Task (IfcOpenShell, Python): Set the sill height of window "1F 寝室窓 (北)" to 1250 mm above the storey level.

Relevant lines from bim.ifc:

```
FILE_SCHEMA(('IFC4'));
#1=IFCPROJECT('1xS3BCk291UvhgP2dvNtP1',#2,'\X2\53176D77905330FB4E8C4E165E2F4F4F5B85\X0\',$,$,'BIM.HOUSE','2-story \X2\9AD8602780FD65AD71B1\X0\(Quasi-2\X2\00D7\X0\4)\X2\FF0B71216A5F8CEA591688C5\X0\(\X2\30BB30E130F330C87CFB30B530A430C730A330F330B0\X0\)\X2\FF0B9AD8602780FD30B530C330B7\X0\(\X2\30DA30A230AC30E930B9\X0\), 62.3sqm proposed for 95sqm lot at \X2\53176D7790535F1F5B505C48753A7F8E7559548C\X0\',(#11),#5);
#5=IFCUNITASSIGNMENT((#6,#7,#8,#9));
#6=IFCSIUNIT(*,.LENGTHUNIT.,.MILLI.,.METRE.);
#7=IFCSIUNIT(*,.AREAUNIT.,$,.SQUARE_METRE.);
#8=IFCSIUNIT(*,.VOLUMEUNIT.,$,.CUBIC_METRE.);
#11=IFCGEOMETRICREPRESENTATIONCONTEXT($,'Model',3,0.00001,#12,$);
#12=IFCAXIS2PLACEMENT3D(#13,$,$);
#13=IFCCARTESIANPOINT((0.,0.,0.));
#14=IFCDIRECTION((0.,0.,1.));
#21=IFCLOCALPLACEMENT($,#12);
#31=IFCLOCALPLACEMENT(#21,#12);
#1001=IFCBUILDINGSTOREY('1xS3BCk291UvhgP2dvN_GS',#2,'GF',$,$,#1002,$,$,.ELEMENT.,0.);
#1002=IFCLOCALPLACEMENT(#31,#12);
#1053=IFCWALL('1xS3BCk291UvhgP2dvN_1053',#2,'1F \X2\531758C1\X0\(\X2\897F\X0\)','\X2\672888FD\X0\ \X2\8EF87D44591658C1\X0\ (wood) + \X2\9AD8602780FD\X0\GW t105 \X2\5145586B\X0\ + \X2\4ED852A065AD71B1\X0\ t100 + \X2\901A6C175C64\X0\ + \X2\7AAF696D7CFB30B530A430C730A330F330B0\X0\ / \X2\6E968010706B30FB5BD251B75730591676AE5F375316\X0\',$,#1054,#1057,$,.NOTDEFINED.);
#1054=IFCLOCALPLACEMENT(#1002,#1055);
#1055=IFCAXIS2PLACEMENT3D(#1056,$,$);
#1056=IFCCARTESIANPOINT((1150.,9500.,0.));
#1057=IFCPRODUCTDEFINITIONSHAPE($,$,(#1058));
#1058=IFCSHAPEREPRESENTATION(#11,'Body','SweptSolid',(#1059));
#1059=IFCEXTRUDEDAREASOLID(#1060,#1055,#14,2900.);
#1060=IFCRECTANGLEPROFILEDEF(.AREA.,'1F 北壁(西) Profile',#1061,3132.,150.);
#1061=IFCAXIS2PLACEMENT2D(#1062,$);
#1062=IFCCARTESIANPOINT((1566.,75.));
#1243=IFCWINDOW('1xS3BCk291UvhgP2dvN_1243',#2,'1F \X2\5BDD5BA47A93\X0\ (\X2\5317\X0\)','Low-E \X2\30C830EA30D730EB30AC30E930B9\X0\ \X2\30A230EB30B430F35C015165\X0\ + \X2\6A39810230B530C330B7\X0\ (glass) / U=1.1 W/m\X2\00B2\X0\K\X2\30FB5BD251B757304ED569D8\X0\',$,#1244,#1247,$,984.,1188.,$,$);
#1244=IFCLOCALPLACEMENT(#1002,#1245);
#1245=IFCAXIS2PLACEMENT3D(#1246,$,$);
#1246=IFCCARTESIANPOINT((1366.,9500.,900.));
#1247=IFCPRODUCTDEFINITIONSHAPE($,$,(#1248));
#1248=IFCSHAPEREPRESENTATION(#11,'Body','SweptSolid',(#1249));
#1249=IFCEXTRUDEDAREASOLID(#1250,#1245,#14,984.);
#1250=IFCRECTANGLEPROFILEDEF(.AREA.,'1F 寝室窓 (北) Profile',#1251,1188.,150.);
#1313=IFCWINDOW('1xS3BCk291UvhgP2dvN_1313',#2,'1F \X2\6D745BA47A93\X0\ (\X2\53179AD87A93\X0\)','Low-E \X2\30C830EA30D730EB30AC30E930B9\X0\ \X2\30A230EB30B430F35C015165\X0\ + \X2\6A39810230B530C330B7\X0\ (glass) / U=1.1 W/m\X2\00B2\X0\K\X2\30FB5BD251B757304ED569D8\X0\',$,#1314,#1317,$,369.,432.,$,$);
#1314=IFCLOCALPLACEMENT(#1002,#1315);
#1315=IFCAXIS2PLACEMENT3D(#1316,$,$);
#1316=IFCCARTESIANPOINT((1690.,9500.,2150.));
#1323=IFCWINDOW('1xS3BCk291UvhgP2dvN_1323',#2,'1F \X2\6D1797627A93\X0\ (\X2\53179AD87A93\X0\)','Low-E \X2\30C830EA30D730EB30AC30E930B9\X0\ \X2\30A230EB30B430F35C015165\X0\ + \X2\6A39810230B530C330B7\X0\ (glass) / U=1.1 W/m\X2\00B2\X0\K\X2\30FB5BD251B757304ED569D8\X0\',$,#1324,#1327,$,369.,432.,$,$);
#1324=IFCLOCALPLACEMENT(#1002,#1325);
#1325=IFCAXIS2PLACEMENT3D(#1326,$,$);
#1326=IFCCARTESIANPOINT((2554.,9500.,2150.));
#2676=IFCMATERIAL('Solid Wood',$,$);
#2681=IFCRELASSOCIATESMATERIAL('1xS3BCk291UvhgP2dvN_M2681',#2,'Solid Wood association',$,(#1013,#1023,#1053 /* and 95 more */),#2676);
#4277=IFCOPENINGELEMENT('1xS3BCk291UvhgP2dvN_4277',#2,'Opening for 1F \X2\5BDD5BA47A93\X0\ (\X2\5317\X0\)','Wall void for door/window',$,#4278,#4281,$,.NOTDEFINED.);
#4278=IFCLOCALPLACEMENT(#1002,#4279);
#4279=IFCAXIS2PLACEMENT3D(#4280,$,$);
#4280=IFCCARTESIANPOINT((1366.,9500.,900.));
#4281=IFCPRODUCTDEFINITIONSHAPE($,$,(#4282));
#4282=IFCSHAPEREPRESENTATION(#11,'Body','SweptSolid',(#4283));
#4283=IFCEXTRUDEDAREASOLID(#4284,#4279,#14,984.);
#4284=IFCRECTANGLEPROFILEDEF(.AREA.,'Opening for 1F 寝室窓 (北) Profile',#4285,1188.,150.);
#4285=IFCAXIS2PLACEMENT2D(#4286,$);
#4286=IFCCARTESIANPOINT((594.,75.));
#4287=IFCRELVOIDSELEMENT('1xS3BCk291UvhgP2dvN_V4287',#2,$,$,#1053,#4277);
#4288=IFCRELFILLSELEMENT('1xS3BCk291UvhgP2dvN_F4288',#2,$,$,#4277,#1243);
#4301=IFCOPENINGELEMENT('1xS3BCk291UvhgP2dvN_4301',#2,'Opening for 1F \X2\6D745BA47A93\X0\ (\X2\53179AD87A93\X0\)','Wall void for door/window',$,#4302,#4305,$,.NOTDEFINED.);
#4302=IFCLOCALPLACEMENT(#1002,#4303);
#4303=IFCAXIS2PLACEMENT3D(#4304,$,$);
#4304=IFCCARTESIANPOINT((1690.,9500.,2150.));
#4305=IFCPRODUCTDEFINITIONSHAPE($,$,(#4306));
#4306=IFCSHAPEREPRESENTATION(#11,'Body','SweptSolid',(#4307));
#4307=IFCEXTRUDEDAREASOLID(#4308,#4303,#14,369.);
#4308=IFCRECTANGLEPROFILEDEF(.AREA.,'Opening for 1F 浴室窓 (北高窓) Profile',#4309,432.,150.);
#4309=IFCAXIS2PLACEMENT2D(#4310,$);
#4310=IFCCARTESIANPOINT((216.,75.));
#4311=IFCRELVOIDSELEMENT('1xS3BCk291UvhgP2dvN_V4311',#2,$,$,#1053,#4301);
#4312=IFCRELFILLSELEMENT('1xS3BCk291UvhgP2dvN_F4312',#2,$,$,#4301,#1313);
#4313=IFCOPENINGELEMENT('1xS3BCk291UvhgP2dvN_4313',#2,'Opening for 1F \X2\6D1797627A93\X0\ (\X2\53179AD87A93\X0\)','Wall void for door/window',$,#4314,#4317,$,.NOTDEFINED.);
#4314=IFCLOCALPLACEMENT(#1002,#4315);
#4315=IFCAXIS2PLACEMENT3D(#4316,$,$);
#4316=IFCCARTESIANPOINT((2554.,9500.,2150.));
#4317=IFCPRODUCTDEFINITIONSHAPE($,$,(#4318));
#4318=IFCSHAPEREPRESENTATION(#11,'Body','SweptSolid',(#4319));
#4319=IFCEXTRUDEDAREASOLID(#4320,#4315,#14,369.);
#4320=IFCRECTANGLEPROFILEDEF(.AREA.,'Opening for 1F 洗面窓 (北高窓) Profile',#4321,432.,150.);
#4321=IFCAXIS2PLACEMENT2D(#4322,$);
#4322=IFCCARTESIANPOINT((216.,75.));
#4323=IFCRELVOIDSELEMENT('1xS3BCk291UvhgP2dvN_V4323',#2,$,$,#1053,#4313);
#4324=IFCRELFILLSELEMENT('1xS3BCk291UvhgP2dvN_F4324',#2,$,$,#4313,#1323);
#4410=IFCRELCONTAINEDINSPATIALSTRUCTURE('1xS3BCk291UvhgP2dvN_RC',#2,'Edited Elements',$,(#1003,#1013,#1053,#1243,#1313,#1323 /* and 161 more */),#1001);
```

```python
import numpy as np
import ifcopenshell
import ifcopenshell.api.geometry
import ifcopenshell.geom
import ifcopenshell.util.element
import ifcopenshell.util.placement
import ifcopenshell.util.shape
import ifcopenshell.util.unit

model = ifcopenshell.open("bim.ifc")
unit_scale = ifcopenshell.util.unit.calculate_unit_scale(model)

window = model.by_id(1243)
opening = window.FillsVoids[0].RelatingOpeningElement
storey = ifcopenshell.util.element.get_container(window, ifc_class="IfcBuildingStorey")
level = ifcopenshell.util.placement.get_local_placement(storey.ObjectPlacement)[2, 3]

# The opening's origin need not be at the sill, so measure its lowest point.
shape = ifcopenshell.geom.create_shape(ifcopenshell.geom.settings(), opening)
bottom = ifcopenshell.util.shape.get_shape_bottom_elevation(shape, shape.geometry) / unit_scale
dz = level + 1.25 / unit_scale - bottom

shift = np.array([0.0, 0.0, dz])
# The window is not placed relative to its opening, so move both.
for product in (opening, window):
    matrix = ifcopenshell.util.placement.get_local_placement(product.ObjectPlacement)
    matrix[:3, 3] += shift
    ifcopenshell.api.geometry.edit_object_placement(model, product=product, matrix=matrix, is_si=False)

print(f"moved by {dz * unit_scale:+.3f} m")

model.write("bim_updated.ifc")
```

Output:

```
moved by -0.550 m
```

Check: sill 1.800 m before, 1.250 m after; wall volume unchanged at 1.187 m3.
